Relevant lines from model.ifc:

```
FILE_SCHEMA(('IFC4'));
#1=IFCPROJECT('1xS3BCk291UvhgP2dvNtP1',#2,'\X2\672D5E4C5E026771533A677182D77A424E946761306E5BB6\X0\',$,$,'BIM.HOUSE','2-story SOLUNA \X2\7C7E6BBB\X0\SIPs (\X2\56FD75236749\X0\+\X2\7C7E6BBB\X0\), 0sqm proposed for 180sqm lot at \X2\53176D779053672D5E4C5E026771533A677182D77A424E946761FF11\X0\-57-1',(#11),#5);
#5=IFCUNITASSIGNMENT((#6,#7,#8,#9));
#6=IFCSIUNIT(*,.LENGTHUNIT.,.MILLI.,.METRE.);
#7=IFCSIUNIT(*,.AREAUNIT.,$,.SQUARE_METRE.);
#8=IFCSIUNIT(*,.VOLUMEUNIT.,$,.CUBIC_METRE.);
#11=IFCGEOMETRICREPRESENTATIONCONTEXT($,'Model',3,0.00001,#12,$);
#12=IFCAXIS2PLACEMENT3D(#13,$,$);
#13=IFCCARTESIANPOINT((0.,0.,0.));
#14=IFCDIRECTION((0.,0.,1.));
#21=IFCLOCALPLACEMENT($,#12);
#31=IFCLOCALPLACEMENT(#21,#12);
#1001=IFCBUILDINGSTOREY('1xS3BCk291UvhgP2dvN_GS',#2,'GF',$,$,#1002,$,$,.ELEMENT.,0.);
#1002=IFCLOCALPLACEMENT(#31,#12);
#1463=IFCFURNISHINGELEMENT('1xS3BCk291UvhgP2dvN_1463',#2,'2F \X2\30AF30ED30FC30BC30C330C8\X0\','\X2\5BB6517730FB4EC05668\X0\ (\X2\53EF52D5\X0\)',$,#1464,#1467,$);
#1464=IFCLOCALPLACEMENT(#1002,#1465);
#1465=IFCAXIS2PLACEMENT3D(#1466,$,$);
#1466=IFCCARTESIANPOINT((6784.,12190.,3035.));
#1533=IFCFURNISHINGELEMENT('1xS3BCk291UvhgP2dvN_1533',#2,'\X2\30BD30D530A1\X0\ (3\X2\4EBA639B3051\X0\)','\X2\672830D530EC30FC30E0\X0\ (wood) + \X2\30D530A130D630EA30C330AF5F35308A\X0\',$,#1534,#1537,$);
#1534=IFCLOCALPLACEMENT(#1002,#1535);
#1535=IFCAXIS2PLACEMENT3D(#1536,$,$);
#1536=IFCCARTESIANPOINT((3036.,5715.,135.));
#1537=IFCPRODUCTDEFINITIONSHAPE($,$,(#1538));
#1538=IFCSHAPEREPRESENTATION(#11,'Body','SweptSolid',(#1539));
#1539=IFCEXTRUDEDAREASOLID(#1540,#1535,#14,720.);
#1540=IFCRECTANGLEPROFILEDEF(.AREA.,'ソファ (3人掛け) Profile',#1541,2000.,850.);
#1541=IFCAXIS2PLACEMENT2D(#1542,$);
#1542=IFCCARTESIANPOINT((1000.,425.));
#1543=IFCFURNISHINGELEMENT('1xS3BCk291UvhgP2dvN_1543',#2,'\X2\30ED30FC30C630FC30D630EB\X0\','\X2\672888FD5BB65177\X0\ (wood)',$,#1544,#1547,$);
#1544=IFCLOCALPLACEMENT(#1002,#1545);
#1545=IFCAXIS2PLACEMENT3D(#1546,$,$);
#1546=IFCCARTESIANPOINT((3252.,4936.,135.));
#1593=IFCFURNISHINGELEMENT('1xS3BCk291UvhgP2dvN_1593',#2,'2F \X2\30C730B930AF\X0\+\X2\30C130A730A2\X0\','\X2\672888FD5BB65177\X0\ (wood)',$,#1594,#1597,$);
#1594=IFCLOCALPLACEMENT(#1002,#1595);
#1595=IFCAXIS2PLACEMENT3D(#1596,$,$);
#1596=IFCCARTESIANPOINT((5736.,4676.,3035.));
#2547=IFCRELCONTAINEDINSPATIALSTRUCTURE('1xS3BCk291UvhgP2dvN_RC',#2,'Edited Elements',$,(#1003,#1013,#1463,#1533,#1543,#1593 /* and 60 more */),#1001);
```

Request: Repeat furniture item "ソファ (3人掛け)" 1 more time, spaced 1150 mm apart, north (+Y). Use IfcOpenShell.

```python
import numpy as np
import ifcopenshell
import ifcopenshell.api.geometry
import ifcopenshell.api.root
import ifcopenshell.util.element
import ifcopenshell.util.placement

model = ifcopenshell.open("model.ifc")


def reuse_history(source, copy):
    """copy_class also copies each property set's owner history, people and application; keep the originals."""
    for rel in copy.IsDefinedBy:
        if rel.is_a("IfcRelDefinesByProperties") and (history := rel.RelatingPropertyDefinition.OwnerHistory):
            rel.RelatingPropertyDefinition.OwnerHistory = source.OwnerHistory
            ifcopenshell.util.element.remove_deep2(model, history)


source = model.by_guid("1xS3BCk291UvhgP2dvN_1533")
base = ifcopenshell.util.placement.get_local_placement(source.ObjectPlacement)
step = np.array([0.0, 1.0, 0.0]) * 1150.0

for i in range(1, 2):
    copy = ifcopenshell.api.root.copy_class(model, product=source)
    copy.Representation = ifcopenshell.util.element.copy_deep(
        model, source.Representation, exclude=["IfcGeometricRepresentationContext", "IfcRepresentationMap"]
    )
    reuse_history(source, copy)
    matrix = base.copy()
    matrix[:3, 3] += i * step
    print("added at", matrix[:3, 3].round(3) + 0.0)
    ifcopenshell.api.geometry.edit_object_placement(model, product=copy, matrix=matrix, is_si=False)

model.write("model_rev.ifc")
```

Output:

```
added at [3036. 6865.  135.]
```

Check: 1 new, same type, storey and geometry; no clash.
